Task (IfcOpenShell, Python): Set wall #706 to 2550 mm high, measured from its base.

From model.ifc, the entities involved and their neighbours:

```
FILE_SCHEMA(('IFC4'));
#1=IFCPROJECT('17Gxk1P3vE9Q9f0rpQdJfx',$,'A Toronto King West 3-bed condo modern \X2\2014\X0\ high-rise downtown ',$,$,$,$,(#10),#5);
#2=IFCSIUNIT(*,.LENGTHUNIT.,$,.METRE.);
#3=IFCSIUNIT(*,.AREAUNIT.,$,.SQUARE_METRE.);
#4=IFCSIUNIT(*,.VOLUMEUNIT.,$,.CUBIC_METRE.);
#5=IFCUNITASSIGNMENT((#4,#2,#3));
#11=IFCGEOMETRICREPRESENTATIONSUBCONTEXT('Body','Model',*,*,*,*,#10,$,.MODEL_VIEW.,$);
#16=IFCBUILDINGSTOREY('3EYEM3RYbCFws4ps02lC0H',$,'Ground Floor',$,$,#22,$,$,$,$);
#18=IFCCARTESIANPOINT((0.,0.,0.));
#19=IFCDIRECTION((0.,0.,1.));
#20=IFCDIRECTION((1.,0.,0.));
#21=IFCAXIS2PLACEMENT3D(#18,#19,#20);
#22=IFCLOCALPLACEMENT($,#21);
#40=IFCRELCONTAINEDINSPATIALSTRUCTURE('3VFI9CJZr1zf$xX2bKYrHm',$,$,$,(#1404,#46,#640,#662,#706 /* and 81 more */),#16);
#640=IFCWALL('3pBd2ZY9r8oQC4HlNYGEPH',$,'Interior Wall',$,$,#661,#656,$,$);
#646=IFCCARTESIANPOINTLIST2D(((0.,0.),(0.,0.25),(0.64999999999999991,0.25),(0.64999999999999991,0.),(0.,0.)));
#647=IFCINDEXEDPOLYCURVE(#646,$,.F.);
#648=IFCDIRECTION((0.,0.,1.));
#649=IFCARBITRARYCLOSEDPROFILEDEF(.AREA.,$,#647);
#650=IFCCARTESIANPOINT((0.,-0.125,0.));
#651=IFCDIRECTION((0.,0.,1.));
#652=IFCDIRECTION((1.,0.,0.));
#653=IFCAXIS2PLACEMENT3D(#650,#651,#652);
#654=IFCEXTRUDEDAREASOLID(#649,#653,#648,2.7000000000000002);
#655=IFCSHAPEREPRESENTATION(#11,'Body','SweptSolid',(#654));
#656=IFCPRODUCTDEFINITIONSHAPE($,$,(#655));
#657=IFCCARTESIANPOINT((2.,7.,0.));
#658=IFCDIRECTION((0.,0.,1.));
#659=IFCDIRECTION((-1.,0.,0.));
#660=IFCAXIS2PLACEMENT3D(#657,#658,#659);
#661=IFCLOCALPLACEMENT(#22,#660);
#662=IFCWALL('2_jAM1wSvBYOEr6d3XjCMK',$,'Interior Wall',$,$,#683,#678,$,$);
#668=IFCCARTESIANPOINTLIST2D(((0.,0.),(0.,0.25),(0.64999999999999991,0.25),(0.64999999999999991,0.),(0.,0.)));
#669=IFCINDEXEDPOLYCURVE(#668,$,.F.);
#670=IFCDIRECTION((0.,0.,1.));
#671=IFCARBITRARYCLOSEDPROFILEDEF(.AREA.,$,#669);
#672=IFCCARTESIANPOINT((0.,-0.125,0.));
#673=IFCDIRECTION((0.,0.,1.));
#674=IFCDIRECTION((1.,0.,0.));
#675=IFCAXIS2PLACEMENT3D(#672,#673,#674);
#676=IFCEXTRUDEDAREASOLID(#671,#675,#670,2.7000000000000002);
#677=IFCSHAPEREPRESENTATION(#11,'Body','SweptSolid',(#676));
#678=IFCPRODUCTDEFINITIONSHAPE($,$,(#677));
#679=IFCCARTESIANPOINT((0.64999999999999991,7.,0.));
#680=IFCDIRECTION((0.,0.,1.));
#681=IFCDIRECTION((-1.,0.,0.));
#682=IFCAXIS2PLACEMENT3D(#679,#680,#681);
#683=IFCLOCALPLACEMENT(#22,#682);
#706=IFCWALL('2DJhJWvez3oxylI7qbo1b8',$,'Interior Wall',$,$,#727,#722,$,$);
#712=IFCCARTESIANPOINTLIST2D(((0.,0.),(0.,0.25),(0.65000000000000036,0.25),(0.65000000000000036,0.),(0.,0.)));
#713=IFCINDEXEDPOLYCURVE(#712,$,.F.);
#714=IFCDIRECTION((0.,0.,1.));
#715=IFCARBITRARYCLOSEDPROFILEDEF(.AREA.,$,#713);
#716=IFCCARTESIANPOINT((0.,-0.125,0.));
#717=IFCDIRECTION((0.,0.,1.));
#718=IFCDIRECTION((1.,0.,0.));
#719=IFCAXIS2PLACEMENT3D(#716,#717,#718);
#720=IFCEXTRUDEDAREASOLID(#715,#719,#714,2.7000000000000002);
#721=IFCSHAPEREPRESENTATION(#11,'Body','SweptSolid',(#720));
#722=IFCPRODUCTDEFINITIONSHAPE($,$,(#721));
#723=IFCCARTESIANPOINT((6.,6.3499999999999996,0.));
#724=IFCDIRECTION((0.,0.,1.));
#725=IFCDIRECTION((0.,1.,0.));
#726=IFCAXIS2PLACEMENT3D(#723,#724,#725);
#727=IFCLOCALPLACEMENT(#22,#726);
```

```python
import ifcopenshell
import ifcopenshell.geom
import ifcopenshell.util.representation
import ifcopenshell.util.shape
import ifcopenshell.util.unit

model = ifcopenshell.open("model.ifc")
unit_scale = ifcopenshell.util.unit.calculate_unit_scale(model)
settings = ifcopenshell.geom.settings()


def volume(element):
    """Net volume in cubic metres, openings subtracted."""
    shape = ifcopenshell.geom.create_shape(settings, element)
    return ifcopenshell.util.shape.get_volume(shape.geometry)


wall = model.by_guid("2DJhJWvez3oxylI7qbo1b8")
before = volume(wall)

body = ifcopenshell.util.representation.get_representation(wall, "Model", "Body")
solid = body.Items[0]
old_height = solid.Depth
solid.Depth = 2.55 / unit_scale
after = volume(wall)

print(f"height {old_height:g} -> {solid.Depth:g}, volume {before:.3f} -> {after:.3f} m3")

model.write("model_edited.ifc")
```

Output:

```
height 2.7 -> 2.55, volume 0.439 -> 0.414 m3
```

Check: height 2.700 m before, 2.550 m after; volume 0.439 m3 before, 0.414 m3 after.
